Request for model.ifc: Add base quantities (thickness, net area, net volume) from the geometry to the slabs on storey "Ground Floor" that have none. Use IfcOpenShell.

First a look at what the model holds.

```python
import ifcopenshell
import ifcopenshell.util.element
import ifcopenshell.util.unit

model = ifcopenshell.open("model.ifc")
print(model.schema)
for unit_type in ("LENGTHUNIT", "AREAUNIT", "VOLUMEUNIT"):
    print(unit_type, ifcopenshell.util.unit.calculate_unit_scale(model, unit_type))
storey = next(s for s in model.by_type("IfcBuildingStorey") if s.Name == "Ground Floor")
slabs = [e for e in ifcopenshell.util.element.get_decomposition(storey) if e.is_a("IfcSlab")]
for e in sorted(slabs, key=lambda e: e.id()):
    print(e.id(), e.is_a(), e.Name, list(ifcopenshell.util.element.get_psets(e, qtos_only=True)), sep=" | ")
```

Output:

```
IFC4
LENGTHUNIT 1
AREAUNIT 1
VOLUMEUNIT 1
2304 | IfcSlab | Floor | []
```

```python
import ifcopenshell
import ifcopenshell.api.pset
import ifcopenshell.geom
import ifcopenshell.util.element
import ifcopenshell.util.shape
import ifcopenshell.util.unit

model = ifcopenshell.open("model.ifc")
unit_scale = ifcopenshell.util.unit.calculate_unit_scale(model)
area_scale = ifcopenshell.util.unit.calculate_unit_scale(model, "AREAUNIT")
volume_scale = ifcopenshell.util.unit.calculate_unit_scale(model, "VOLUMEUNIT")
settings = ifcopenshell.geom.settings()

storey = next(s for s in model.by_type("IfcBuildingStorey") if s.Name == "Ground Floor")
slabs = [e for e in ifcopenshell.util.element.get_decomposition(storey) if e.is_a("IfcSlab")]

for e in sorted(slabs, key=lambda e: e.id()):
    if ifcopenshell.util.element.get_psets(e, qtos_only=True, should_inherit=False):
        continue
    # Geometry comes back in metres, in the element's own axes.
    shape = ifcopenshell.geom.create_shape(settings, e)
    values = {
        "Width": ifcopenshell.util.shape.get_z(shape.geometry) / unit_scale,
        "NetArea": ifcopenshell.util.shape.get_footprint_area(shape.geometry) / area_scale,
        "NetVolume": ifcopenshell.util.shape.get_volume(shape.geometry) / volume_scale,
    }
    qto = ifcopenshell.api.pset.add_qto(model, product=e, name="Qto_SlabBaseQuantities")
    ifcopenshell.api.pset.edit_qto(model, qto=qto, properties=values)
    print(e.id(), {k: round(v, 3) for k, v in values.items()})

model.write("model_v2.ifc")
```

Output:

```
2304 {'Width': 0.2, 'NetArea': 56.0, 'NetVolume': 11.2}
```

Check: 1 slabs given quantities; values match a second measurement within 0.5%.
